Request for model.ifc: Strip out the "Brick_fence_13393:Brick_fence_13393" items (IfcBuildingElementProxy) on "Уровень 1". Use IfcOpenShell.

First a look at what the model holds.

```python
import ifcopenshell
import ifcopenshell.util.element

model = ifcopenshell.open("model.ifc")
print(model.schema)
storey = next(s for s in model.by_type("IfcBuildingStorey") if s.Name == "Уровень 1")
proxies = [e for e in ifcopenshell.util.element.get_decomposition(storey) if e.is_a("IfcBuildingElementProxy")]
seen = {}
for e in proxies:
    element_type = ifcopenshell.util.element.get_type(e)
    name = element_type.Name if element_type not in (None, e) else None
    seen[name] = seen.get(name, 0) + 1
for name, count in sorted(seen.items(), key=str):
    print(count, "x", name)
```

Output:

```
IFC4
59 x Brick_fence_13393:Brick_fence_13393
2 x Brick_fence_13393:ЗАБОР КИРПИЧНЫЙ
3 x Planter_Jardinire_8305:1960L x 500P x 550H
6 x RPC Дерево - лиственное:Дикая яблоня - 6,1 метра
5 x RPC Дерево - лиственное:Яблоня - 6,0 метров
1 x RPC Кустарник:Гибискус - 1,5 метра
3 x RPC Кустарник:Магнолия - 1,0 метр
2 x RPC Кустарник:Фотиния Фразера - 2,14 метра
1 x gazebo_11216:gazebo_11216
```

```python
import ifcopenshell
import ifcopenshell.api.root
import ifcopenshell.util.element

model = ifcopenshell.open("model.ifc")

storey = next(s for s in model.by_type("IfcBuildingStorey") if s.Name == "Уровень 1")
proxies = [e for e in ifcopenshell.util.element.get_decomposition(storey) if e.is_a("IfcBuildingElementProxy")]
targets = [e for e in proxies if (t := ifcopenshell.util.element.get_type(e)) not in (None, e) and t.Name == "Brick_fence_13393:Brick_fence_13393"]

for e in targets:
    ifcopenshell.api.root.remove_product(model, product=e)
print(len(targets), "removed")

model.write("model_rev.ifc")
```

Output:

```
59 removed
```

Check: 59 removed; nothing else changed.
